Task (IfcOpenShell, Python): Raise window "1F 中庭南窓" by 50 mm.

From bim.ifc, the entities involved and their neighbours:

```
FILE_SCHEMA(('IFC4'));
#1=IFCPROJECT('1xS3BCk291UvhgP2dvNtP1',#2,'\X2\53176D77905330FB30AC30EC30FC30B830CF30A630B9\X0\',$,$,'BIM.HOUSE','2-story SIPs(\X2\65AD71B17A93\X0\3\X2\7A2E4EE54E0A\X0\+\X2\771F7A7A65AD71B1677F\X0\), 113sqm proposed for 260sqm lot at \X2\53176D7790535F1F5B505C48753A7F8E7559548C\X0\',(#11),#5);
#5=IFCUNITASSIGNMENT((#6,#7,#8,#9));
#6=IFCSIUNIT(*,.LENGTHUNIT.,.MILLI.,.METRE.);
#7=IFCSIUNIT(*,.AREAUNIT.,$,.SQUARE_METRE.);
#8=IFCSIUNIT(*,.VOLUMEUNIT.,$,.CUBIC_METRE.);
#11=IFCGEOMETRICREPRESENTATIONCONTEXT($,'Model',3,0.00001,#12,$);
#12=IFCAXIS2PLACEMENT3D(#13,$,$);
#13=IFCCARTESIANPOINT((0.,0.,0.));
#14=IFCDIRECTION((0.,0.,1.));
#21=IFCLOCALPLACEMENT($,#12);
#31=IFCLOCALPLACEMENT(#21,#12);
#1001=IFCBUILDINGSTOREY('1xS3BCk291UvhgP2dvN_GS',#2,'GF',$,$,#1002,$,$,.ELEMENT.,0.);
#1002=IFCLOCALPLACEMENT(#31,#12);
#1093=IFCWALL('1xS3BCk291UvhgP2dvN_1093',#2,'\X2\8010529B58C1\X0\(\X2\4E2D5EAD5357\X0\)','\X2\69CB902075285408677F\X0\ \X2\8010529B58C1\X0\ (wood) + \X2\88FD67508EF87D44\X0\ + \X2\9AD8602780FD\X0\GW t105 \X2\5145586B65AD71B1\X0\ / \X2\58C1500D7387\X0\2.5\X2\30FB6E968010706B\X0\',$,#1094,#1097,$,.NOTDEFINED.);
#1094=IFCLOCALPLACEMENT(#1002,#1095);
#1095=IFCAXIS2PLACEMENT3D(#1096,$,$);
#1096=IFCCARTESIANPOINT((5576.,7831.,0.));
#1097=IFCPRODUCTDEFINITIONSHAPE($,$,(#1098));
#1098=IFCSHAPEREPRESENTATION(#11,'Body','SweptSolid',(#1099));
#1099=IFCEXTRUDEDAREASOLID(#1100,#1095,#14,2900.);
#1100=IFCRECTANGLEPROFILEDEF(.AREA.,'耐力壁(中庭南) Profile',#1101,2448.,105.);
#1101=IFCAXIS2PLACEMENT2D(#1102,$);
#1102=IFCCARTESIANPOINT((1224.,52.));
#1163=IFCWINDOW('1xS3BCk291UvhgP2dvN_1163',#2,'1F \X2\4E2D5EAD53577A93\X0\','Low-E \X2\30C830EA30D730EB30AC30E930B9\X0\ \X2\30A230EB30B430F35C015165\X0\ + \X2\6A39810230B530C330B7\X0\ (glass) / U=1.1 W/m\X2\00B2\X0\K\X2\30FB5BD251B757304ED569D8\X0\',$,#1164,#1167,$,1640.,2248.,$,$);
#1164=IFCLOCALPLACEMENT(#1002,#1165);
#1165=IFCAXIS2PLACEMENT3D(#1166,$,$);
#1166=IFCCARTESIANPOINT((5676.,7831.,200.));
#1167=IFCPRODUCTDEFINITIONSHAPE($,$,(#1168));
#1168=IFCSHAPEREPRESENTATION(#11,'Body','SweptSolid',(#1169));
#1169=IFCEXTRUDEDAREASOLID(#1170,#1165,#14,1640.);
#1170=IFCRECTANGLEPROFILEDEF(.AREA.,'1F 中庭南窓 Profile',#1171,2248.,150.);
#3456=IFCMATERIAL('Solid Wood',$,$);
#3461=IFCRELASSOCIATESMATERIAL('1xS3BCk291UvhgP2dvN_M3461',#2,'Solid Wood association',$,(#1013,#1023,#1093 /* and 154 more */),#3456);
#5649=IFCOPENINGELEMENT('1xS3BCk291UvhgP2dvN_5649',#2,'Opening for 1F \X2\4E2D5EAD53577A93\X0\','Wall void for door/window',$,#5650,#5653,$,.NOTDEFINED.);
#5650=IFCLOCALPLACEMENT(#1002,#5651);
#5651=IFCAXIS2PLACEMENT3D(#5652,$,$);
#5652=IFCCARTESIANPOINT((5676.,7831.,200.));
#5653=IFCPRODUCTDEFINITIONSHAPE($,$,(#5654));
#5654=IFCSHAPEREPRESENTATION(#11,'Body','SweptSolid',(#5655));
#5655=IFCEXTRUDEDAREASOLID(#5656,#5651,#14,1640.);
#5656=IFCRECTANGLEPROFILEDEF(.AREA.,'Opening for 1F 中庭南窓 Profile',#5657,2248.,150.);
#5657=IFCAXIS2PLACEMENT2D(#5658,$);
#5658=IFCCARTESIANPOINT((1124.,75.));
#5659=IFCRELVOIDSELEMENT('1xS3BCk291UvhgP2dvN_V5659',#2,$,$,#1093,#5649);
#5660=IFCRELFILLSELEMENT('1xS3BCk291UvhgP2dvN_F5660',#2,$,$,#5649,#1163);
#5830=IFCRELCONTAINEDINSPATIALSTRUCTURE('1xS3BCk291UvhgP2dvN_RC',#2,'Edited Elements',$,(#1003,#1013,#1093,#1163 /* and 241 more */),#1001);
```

```python
import numpy as np
import ifcopenshell
import ifcopenshell.api.geometry
import ifcopenshell.util.placement
import ifcopenshell.util.unit

model = ifcopenshell.open("bim.ifc")
unit_scale = ifcopenshell.util.unit.calculate_unit_scale(model)

window = model.by_guid("1xS3BCk291UvhgP2dvN_1163")
opening = window.FillsVoids[0].RelatingOpeningElement
dz = 50.0

shift = np.array([0.0, 0.0, dz])
# The window is not placed relative to its opening, so move both.
for product in (opening, window):
    matrix = ifcopenshell.util.placement.get_local_placement(product.ObjectPlacement)
    matrix[:3, 3] += shift
    ifcopenshell.api.geometry.edit_object_placement(model, product=product, matrix=matrix, is_si=False)

print(f"moved by {dz * unit_scale:+.3f} m")

model.write("bim_rev.ifc")
```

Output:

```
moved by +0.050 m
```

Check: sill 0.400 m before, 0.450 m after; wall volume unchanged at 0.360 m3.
